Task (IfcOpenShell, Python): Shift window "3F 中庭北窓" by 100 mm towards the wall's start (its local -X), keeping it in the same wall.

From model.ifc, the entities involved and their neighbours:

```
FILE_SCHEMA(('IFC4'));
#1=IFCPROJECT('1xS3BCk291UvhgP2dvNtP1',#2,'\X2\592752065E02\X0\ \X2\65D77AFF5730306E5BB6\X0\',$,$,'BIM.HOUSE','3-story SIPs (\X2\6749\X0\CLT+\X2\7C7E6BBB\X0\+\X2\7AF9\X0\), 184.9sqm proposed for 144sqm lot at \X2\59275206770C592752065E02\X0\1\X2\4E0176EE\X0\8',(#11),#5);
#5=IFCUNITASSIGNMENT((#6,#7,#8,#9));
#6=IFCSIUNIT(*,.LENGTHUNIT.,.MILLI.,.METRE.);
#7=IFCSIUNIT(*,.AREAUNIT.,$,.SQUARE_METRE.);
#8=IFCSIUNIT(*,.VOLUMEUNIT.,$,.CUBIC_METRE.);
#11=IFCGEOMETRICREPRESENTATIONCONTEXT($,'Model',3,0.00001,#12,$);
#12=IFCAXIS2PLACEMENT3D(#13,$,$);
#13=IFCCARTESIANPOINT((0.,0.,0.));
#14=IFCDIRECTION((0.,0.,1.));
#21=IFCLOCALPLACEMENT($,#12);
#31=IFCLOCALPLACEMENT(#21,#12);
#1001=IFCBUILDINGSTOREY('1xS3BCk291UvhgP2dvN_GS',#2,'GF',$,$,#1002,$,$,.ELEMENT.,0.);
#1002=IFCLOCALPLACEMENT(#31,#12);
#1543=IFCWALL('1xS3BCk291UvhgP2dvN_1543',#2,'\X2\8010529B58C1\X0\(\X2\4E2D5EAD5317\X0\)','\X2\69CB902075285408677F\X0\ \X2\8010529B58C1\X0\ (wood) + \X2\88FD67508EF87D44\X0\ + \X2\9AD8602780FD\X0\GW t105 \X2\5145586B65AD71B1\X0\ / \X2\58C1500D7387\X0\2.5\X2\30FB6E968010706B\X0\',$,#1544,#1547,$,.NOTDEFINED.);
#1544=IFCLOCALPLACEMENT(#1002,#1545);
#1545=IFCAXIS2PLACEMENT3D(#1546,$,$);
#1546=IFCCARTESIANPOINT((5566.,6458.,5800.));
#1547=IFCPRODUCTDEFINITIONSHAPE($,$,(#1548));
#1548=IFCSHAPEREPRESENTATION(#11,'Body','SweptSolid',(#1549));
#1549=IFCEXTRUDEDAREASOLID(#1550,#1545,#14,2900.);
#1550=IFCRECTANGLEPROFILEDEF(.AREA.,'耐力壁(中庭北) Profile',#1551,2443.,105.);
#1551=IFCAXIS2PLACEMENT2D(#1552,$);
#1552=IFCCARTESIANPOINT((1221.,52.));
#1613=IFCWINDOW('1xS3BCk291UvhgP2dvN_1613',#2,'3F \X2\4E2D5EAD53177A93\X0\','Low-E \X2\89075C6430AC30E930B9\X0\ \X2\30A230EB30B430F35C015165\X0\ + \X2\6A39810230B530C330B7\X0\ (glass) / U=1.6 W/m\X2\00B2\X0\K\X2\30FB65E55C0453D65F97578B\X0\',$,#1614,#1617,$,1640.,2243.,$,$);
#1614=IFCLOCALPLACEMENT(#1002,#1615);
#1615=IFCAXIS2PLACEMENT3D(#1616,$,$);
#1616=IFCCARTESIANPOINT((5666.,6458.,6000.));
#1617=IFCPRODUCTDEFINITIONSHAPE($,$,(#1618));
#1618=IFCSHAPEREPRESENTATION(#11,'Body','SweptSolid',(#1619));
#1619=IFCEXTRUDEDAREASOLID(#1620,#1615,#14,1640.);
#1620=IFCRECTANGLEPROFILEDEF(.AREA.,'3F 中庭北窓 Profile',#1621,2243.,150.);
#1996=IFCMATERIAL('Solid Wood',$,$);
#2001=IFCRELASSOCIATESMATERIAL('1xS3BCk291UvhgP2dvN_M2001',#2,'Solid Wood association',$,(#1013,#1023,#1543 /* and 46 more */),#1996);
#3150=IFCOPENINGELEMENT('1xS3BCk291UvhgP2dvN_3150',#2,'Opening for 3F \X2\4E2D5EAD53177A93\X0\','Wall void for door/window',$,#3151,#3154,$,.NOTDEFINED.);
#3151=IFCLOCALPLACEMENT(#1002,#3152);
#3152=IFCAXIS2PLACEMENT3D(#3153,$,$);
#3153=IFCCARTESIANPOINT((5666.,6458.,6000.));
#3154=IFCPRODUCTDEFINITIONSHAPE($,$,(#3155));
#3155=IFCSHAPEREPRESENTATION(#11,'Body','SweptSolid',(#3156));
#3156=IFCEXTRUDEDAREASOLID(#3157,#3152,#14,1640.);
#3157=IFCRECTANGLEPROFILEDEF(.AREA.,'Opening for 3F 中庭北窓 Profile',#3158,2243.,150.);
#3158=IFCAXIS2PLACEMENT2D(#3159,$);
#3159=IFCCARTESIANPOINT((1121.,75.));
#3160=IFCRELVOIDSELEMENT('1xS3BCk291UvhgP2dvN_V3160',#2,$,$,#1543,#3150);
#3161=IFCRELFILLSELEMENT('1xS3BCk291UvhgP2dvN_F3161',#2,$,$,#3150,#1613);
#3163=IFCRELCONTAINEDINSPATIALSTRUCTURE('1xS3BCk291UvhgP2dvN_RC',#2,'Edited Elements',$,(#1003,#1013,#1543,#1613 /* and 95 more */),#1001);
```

```python
import ifcopenshell
import ifcopenshell.api.geometry
import ifcopenshell.util.placement
import ifcopenshell.util.unit

model = ifcopenshell.open("model.ifc")
unit_scale = ifcopenshell.util.unit.calculate_unit_scale(model)

window = model.by_guid("1xS3BCk291UvhgP2dvN_1613")
opening = window.FillsVoids[0].RelatingOpeningElement
wall = opening.VoidsElements[0].RelatingBuildingElement

wall_matrix = ifcopenshell.util.placement.get_local_placement(wall.ObjectPlacement)
shift = wall_matrix[:3, 0] * -0.1 / unit_scale
before = ifcopenshell.util.placement.get_local_placement(window.ObjectPlacement)[:3, 3].copy()

# The window is not placed relative to its opening, so move both.
for product in (opening, window):
    matrix = ifcopenshell.util.placement.get_local_placement(product.ObjectPlacement)
    matrix[:3, 3] += shift
    ifcopenshell.api.geometry.edit_object_placement(model, product=product, matrix=matrix, is_si=False)

after = ifcopenshell.util.placement.get_local_placement(window.ObjectPlacement)[:3, 3]
print("window moved by", (after - before).round(3) + 0.0)

model.write("model_updated.ifc")
```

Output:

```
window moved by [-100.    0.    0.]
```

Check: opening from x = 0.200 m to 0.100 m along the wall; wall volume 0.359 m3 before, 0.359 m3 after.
